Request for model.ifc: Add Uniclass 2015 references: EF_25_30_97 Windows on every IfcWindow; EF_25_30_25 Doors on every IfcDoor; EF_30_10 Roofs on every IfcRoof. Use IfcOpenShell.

First a look at what the model holds.

```python
import ifcopenshell

model = ifcopenshell.open("model.ifc")
print(model.schema)
print("classifications:", [c.Name for c in model.by_type("IfcClassification")])
for ifc_class in ("IfcDoor", "IfcRoof", "IfcStair", "IfcWall", "IfcWindow"):
    print(ifc_class, len(model.by_type(ifc_class)))
```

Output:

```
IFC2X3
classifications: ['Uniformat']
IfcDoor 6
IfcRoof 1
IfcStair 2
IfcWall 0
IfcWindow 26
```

```python
import ifcopenshell
import ifcopenshell.api.classification

model = ifcopenshell.open("model.ifc")

# IFC2X3 requires Source and Edition and has no link from the project to the system.
system = model.create_entity("IfcClassification", Source="NBS", Edition="2015", Name="Uniclass 2015")

codes = {
    "IfcWindow": ("EF_25_30_97", "Windows"),
    "IfcDoor": ("EF_25_30_25", "Doors"),
    "IfcRoof": ("EF_30_10", "Roofs"),
}
for ifc_class, (code, name) in codes.items():
    products = model.by_type(ifc_class)
    ifcopenshell.api.classification.add_reference(
        model, products=products, classification=system, identification=code, name=name
    )
    print(code, len(products))

model.write("model_edited.ifc")
```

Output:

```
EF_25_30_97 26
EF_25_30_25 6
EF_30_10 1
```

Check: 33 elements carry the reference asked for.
